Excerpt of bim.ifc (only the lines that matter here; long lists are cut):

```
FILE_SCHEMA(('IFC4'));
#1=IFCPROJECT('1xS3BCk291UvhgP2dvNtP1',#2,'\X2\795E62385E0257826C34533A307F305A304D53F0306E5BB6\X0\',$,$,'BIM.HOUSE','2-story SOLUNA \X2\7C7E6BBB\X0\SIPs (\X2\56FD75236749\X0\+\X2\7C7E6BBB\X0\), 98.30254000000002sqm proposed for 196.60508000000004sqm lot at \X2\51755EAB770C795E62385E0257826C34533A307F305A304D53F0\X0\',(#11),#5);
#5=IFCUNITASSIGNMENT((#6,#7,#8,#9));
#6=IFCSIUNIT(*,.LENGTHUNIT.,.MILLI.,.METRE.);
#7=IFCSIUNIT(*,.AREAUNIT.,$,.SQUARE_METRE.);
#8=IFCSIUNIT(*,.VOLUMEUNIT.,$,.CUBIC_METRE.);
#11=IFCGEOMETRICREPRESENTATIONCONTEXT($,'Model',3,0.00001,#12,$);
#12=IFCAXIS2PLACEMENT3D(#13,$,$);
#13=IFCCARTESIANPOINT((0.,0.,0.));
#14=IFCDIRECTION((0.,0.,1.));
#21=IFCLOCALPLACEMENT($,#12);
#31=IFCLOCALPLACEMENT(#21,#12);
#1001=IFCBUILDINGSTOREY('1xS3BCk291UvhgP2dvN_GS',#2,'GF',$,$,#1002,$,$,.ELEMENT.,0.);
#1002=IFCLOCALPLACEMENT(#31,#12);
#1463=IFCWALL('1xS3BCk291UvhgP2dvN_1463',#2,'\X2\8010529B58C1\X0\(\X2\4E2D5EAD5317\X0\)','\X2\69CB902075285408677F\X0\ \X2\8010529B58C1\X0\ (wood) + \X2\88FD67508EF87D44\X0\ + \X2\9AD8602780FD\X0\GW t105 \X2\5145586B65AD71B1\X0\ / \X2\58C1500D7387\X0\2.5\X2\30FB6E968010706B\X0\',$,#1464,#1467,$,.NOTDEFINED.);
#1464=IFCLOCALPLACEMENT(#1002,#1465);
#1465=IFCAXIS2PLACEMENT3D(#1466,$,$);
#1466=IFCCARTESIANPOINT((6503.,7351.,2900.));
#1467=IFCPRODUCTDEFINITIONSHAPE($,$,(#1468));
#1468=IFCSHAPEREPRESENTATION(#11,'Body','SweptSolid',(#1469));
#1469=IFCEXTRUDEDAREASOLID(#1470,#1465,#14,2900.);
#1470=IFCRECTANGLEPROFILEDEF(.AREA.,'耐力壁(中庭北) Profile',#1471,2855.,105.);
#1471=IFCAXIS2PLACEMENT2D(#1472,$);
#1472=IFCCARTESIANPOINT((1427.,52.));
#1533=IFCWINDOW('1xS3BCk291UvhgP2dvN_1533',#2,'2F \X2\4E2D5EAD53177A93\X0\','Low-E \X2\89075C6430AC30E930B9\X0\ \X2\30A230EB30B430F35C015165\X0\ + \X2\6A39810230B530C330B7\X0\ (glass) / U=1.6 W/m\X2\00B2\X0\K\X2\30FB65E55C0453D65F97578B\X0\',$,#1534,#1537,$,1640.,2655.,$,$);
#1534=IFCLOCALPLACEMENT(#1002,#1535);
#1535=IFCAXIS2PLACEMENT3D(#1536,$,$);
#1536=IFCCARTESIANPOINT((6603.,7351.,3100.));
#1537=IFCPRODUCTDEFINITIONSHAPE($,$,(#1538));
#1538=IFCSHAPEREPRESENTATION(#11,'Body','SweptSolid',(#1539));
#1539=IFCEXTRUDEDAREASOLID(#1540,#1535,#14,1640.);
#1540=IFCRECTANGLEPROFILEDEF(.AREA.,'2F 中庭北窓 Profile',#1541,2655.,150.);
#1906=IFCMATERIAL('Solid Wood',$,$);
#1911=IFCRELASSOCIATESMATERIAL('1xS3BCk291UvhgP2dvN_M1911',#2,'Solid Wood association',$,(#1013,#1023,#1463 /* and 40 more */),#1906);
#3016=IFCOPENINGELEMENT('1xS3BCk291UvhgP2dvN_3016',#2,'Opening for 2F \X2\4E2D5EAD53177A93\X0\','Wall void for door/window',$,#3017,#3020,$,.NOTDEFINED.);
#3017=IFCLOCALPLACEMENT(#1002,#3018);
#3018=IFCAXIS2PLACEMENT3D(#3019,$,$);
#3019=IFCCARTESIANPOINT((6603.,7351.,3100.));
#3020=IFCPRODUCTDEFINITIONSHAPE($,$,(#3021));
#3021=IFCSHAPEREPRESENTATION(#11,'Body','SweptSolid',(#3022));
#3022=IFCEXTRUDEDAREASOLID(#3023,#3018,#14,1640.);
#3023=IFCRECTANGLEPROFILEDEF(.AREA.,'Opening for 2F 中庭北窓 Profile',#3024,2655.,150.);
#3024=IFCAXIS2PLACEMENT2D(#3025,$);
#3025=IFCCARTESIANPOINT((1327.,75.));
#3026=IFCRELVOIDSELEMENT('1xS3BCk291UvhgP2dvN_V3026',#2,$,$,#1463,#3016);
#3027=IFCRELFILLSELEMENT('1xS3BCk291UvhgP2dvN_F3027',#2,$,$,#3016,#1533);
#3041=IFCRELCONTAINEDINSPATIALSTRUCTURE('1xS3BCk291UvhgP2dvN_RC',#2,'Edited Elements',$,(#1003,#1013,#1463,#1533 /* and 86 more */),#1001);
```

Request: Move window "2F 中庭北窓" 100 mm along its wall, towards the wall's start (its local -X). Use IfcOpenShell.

```python
import ifcopenshell
import ifcopenshell.api.geometry
import ifcopenshell.util.placement

model = ifcopenshell.open("bim.ifc")

window = model.by_guid("1xS3BCk291UvhgP2dvN_1533")
opening = window.FillsVoids[0].RelatingOpeningElement
wall = opening.VoidsElements[0].RelatingBuildingElement

wall_matrix = ifcopenshell.util.placement.get_local_placement(wall.ObjectPlacement)
shift = wall_matrix[:3, 0] * -100.0
before = ifcopenshell.util.placement.get_local_placement(window.ObjectPlacement)[:3, 3].copy()

# The window is not placed relative to its opening, so move both.
for product in (opening, window):
    matrix = ifcopenshell.util.placement.get_local_placement(product.ObjectPlacement)
    matrix[:3, 3] += shift
    ifcopenshell.api.geometry.edit_object_placement(model, product=product, matrix=matrix, is_si=False)

after = ifcopenshell.util.placement.get_local_placement(window.ObjectPlacement)[:3, 3]
print("window moved by", (after - before).round(3) + 0.0)

model.write("bim_v2.ifc")
```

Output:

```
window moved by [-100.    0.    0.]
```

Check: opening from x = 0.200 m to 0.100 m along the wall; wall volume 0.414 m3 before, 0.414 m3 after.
